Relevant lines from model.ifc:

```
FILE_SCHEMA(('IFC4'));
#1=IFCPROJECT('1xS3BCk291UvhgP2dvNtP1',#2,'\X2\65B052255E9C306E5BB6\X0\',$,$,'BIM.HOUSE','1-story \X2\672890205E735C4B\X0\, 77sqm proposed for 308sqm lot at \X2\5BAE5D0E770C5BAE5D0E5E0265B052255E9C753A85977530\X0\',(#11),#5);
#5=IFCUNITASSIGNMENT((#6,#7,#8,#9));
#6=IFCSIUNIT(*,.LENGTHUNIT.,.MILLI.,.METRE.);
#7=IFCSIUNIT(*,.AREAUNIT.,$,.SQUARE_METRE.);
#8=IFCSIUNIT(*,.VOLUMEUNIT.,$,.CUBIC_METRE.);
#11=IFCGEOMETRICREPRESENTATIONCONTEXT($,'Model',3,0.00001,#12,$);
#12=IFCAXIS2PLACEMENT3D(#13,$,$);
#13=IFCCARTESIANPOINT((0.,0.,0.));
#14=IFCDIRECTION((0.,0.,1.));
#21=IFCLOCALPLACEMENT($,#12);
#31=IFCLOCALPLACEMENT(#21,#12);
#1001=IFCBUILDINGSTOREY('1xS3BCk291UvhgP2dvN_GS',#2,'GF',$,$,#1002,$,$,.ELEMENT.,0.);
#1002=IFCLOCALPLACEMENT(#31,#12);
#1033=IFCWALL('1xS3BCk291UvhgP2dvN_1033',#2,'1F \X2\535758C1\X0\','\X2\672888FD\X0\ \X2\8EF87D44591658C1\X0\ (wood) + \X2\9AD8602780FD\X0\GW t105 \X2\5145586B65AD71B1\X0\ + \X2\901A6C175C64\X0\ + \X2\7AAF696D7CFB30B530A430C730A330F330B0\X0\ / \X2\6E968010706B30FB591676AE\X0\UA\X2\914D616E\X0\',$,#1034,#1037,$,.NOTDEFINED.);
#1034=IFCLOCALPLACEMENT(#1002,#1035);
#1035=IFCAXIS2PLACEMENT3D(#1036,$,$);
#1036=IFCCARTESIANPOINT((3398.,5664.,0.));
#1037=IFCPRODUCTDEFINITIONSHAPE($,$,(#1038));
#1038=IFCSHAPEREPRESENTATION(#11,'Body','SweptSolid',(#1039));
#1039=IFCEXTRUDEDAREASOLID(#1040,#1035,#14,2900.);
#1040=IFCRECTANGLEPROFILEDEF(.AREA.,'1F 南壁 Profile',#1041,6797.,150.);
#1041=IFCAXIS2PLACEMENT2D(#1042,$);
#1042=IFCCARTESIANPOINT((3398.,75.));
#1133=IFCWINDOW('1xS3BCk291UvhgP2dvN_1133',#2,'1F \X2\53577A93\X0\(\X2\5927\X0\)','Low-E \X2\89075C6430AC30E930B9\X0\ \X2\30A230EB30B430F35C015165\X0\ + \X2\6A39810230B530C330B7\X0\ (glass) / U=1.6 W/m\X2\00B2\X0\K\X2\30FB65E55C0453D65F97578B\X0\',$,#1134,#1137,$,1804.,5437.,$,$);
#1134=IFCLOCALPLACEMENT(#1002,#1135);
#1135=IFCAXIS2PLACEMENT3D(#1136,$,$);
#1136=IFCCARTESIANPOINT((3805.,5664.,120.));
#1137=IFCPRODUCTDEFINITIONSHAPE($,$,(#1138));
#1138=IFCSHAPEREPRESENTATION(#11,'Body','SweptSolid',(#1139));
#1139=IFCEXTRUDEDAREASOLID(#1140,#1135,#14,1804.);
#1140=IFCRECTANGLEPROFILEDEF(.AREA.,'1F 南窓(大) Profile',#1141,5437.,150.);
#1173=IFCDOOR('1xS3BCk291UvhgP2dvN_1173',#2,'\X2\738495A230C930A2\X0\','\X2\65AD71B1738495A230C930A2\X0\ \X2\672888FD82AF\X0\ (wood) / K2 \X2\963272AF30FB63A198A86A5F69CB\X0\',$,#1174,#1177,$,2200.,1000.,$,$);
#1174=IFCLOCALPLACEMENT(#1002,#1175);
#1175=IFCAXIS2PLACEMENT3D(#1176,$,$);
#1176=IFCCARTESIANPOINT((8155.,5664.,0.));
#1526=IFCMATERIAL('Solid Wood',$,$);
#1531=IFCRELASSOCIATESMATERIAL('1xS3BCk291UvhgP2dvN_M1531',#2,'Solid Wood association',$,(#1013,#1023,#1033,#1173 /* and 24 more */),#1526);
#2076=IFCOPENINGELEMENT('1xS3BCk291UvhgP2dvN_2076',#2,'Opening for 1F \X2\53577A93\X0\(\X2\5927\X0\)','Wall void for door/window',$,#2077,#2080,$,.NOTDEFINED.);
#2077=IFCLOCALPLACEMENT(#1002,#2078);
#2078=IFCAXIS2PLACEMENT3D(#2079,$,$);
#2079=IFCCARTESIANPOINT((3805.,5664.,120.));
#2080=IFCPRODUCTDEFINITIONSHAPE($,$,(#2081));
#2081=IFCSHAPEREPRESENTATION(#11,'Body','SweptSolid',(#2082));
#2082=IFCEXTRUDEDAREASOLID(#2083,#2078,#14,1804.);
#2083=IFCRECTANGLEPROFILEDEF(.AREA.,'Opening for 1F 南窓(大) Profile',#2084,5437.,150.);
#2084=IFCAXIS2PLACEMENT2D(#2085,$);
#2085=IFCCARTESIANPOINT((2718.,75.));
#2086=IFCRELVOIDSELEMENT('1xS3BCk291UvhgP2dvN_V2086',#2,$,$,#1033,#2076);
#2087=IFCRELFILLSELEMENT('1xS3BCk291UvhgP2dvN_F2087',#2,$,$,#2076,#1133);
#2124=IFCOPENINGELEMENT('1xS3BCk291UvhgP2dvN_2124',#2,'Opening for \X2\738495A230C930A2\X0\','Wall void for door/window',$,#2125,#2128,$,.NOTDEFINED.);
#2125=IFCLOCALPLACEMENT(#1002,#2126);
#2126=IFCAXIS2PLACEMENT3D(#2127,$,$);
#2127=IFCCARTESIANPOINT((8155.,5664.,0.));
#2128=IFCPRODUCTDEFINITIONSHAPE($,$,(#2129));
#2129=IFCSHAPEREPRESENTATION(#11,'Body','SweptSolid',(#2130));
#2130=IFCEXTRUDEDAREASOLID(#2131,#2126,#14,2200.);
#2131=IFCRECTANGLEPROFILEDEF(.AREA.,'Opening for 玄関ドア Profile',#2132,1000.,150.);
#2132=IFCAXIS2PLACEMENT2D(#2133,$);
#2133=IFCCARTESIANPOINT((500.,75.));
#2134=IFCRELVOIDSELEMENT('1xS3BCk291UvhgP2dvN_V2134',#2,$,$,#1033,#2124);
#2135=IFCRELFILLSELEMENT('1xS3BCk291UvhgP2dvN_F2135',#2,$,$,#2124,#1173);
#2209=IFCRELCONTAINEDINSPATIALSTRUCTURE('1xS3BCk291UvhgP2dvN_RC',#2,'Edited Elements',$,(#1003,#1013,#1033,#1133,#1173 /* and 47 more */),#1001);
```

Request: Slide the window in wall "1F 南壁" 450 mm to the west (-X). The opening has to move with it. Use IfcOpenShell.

```python
import ifcopenshell
import ifcopenshell.api.geometry
import ifcopenshell.util.placement
import ifcopenshell.util.unit

model = ifcopenshell.open("model.ifc")
unit_scale = ifcopenshell.util.unit.calculate_unit_scale(model)

window = model.by_guid("1xS3BCk291UvhgP2dvN_1133")
opening = window.FillsVoids[0].RelatingOpeningElement
wall = opening.VoidsElements[0].RelatingBuildingElement

wall_matrix = ifcopenshell.util.placement.get_local_placement(wall.ObjectPlacement)
shift = wall_matrix[:3, 0] * -0.45 / unit_scale
before = ifcopenshell.util.placement.get_local_placement(window.ObjectPlacement)[:3, 3].copy()

# The window is not placed relative to its opening, so move both.
for product in (opening, window):
    matrix = ifcopenshell.util.placement.get_local_placement(product.ObjectPlacement)
    matrix[:3, 3] += shift
    ifcopenshell.api.geometry.edit_object_placement(model, product=product, matrix=matrix, is_si=False)

after = ifcopenshell.util.placement.get_local_placement(window.ObjectPlacement)[:3, 3]
print("window moved by", (after - before).round(3) + 0.0)

model.write("model_edited.ifc")
```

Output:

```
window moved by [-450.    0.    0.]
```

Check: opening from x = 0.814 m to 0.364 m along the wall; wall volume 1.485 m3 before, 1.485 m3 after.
